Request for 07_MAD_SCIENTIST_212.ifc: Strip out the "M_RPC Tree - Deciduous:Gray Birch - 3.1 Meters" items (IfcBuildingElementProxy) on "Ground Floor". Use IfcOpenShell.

First a look at what the model holds.

```python
import ifcopenshell
import ifcopenshell.util.element

model = ifcopenshell.open("07_MAD_SCIENTIST_212.ifc")
print(model.schema)
storey = next(s for s in model.by_type("IfcBuildingStorey") if s.Name == "Ground Floor")
proxies = [e for e in ifcopenshell.util.element.get_decomposition(storey) if e.is_a("IfcBuildingElementProxy")]
seen = {}
for e in proxies:
    element_type = ifcopenshell.util.element.get_type(e)
    name = element_type.Name if element_type not in (None, e) else None
    seen[name] = seen.get(name, 0) + 1
for name, count in sorted(seen.items(), key=str):
    print(count, "x", name)
```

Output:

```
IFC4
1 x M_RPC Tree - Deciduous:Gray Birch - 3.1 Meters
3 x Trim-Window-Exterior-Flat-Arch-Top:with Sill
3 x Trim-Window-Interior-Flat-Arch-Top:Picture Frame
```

```python
import ifcopenshell
import ifcopenshell.api.root
import ifcopenshell.util.element

model = ifcopenshell.open("07_MAD_SCIENTIST_212.ifc")

storey = next(s for s in model.by_type("IfcBuildingStorey") if s.Name == "Ground Floor")
proxies = [e for e in ifcopenshell.util.element.get_decomposition(storey) if e.is_a("IfcBuildingElementProxy")]
targets = [e for e in proxies if (t := ifcopenshell.util.element.get_type(e)) not in (None, e) and t.Name == "M_RPC Tree - Deciduous:Gray Birch - 3.1 Meters"]

for e in targets:
    ifcopenshell.api.root.remove_product(model, product=e)
print(len(targets), "removed")

model.write("07_MAD_SCIENTIST_212_updated.ifc")
```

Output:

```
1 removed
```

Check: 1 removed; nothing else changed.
